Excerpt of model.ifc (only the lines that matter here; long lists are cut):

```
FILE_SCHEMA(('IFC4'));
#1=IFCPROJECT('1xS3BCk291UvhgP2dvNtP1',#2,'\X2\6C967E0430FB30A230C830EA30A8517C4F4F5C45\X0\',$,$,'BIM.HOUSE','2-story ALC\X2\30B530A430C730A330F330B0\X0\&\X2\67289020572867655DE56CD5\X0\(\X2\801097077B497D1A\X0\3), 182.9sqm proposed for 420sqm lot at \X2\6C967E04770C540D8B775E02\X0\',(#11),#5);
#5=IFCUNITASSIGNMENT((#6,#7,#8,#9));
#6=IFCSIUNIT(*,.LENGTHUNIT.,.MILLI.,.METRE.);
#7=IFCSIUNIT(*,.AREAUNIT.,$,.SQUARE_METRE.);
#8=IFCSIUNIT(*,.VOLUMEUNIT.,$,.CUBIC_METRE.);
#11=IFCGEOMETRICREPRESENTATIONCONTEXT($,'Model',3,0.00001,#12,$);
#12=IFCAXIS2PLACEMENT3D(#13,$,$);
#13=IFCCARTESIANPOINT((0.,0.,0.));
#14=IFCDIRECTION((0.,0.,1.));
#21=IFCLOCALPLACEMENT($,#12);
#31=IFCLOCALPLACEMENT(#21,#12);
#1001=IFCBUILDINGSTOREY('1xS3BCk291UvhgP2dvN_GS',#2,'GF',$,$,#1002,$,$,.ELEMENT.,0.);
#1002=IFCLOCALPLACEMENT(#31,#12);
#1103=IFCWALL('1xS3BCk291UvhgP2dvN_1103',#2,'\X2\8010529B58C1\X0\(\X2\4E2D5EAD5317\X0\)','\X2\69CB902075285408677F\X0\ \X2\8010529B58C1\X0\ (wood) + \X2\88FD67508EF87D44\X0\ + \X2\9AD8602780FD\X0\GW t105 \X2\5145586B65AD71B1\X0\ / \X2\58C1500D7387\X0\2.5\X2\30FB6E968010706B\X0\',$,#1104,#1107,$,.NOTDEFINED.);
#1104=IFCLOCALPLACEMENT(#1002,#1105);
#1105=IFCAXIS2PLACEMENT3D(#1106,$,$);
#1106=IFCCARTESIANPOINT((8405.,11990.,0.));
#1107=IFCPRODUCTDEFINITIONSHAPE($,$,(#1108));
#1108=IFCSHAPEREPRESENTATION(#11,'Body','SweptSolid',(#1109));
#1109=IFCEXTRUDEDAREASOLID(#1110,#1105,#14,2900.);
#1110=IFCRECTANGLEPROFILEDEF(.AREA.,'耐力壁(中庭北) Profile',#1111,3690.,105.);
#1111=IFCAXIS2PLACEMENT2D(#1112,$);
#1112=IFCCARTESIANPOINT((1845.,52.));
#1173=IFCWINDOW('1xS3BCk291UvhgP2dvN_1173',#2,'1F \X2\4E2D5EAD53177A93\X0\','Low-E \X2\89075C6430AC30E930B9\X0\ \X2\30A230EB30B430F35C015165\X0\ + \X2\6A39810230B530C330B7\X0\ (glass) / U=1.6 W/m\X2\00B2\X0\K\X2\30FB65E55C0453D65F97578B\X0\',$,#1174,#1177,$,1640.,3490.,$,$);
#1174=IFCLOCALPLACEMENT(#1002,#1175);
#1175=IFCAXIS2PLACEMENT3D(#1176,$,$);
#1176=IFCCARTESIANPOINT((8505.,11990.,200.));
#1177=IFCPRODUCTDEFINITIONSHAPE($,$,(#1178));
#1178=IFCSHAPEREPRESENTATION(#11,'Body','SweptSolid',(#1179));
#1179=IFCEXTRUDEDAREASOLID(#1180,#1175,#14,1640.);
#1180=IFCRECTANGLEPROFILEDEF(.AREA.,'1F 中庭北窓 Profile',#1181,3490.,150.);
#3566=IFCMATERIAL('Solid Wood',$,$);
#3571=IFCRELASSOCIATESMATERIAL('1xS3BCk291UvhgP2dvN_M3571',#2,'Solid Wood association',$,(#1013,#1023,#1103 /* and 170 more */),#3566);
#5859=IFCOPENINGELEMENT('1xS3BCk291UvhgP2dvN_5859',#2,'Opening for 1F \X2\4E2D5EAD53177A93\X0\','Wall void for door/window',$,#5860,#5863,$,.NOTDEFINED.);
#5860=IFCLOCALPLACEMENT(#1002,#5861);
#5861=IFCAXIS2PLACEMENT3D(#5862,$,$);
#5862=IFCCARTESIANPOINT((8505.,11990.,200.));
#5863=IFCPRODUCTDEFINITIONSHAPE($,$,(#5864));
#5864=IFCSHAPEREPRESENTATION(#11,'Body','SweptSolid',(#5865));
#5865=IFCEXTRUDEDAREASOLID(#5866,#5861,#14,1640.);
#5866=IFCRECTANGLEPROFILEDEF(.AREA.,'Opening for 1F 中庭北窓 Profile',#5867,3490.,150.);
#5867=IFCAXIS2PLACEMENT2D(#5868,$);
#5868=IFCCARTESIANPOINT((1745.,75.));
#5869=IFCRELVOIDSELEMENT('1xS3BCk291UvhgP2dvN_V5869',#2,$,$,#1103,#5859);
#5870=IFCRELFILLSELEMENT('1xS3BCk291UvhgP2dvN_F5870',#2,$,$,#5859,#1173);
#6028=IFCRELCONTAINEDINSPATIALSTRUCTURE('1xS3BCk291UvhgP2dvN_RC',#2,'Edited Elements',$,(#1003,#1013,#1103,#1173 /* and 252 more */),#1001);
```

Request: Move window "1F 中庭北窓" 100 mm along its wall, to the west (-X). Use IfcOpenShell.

```python
import ifcopenshell
import ifcopenshell.api.geometry
import ifcopenshell.util.placement
import ifcopenshell.util.unit

model = ifcopenshell.open("model.ifc")
unit_scale = ifcopenshell.util.unit.calculate_unit_scale(model)

window = model.by_id(1173)
opening = window.FillsVoids[0].RelatingOpeningElement
wall = opening.VoidsElements[0].RelatingBuildingElement

wall_matrix = ifcopenshell.util.placement.get_local_placement(wall.ObjectPlacement)
shift = wall_matrix[:3, 0] * -0.1 / unit_scale
before = ifcopenshell.util.placement.get_local_placement(window.ObjectPlacement)[:3, 3].copy()

# The window is not placed relative to its opening, so move both.
for product in (opening, window):
    matrix = ifcopenshell.util.placement.get_local_placement(product.ObjectPlacement)
    matrix[:3, 3] += shift
    ifcopenshell.api.geometry.edit_object_placement(model, product=product, matrix=matrix, is_si=False)

after = ifcopenshell.util.placement.get_local_placement(window.ObjectPlacement)[:3, 3]
print("window moved by", (after - before).round(3) + 0.0)

model.write("model_updated.ifc")
```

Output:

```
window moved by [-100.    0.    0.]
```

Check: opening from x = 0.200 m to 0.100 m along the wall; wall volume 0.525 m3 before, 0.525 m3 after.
